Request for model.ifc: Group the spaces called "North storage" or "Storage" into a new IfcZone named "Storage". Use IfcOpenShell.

First a look at what the model holds.

```python
import ifcopenshell

model = ifcopenshell.open("model.ifc")
print(model.schema)
seen = {}
for space in model.by_type("IfcSpace"):
    seen[space.LongName] = seen.get(space.LongName, 0) + 1
for name, count in sorted(seen.items(), key=str):
    print(count, "x", name)
print("zones:", [z.Name for z in model.by_type("IfcZone")][:20])
```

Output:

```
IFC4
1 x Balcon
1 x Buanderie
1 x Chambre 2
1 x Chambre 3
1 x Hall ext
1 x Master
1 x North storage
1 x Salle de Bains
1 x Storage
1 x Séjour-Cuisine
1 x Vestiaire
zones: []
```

```python
import ifcopenshell
import ifcopenshell.api.group
import ifcopenshell.api.root

model = ifcopenshell.open("model.ifc")

names = {"North storage", "Storage"}
spaces = [s for s in model.by_type("IfcSpace") if s.LongName in names]

zone = ifcopenshell.api.root.create_entity(model, ifc_class="IfcZone", name="Storage")
ifcopenshell.api.group.assign_group(model, products=spaces, group=zone)
print(len(spaces), "spaces in", zone.Name)

model.write("model_edited.ifc")
```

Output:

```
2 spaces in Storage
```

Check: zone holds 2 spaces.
